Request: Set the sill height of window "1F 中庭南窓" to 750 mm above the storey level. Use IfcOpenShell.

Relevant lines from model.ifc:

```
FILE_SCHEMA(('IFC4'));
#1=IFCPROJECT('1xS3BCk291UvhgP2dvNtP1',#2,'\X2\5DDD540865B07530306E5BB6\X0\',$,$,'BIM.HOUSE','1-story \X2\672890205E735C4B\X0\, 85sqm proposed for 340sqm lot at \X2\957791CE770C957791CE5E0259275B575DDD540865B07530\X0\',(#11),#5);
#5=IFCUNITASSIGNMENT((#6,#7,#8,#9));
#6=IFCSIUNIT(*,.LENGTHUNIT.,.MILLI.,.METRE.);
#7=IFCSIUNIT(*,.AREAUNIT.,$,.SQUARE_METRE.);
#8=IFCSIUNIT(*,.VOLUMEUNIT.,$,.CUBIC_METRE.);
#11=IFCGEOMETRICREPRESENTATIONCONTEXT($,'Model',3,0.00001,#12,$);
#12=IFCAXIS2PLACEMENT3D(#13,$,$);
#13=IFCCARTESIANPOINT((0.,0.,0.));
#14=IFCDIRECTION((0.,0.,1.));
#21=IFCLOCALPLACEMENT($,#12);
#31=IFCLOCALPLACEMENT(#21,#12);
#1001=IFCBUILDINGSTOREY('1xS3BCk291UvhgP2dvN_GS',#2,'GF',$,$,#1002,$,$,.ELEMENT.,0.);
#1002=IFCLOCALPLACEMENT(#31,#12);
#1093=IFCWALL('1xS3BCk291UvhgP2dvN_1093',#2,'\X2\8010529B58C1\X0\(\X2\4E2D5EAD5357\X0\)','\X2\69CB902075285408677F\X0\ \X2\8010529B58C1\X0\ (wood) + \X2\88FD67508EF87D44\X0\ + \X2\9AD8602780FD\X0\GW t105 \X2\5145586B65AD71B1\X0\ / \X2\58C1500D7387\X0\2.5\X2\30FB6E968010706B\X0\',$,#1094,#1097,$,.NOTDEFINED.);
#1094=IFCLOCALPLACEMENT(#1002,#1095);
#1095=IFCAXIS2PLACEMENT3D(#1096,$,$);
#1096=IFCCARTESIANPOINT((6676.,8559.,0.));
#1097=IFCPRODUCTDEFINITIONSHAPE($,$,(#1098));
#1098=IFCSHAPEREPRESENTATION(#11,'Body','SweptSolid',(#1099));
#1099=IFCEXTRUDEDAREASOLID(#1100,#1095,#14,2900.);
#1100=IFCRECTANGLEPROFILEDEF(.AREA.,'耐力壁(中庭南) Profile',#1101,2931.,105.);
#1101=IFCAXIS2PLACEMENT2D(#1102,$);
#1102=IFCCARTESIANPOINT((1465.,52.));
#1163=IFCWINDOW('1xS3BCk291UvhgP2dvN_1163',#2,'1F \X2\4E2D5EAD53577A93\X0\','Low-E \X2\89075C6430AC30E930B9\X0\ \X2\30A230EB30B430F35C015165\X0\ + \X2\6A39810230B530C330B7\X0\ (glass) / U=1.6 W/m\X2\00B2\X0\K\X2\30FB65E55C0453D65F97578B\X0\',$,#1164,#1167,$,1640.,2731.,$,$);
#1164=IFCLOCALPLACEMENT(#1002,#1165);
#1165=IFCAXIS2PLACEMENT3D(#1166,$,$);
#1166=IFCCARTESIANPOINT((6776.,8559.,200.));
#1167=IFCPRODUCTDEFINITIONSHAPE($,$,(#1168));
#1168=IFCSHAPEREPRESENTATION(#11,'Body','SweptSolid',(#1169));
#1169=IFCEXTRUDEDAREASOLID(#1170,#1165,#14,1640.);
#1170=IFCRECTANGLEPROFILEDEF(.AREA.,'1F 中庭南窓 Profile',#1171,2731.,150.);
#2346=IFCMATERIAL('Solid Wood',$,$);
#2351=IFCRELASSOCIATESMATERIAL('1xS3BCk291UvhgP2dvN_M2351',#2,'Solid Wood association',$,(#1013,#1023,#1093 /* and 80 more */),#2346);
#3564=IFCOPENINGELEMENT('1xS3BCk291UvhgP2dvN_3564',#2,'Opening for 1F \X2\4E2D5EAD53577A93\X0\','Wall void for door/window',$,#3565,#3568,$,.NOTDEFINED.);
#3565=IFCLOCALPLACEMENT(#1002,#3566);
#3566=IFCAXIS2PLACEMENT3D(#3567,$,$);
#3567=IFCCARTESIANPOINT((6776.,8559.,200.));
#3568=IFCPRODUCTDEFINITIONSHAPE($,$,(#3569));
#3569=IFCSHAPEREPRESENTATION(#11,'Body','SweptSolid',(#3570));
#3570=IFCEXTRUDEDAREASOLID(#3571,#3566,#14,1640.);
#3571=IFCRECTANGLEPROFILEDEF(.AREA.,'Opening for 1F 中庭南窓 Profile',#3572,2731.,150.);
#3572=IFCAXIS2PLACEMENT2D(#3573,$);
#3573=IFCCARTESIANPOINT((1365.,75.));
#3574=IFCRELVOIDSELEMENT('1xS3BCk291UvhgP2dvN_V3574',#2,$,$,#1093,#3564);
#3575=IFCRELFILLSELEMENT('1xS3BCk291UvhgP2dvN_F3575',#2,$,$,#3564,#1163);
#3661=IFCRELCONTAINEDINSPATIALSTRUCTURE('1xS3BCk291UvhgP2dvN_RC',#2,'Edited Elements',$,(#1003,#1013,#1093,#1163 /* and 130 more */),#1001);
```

```python
import numpy as np
import ifcopenshell
import ifcopenshell.api.geometry
import ifcopenshell.geom
import ifcopenshell.util.element
import ifcopenshell.util.placement
import ifcopenshell.util.shape
import ifcopenshell.util.unit

model = ifcopenshell.open("model.ifc")
unit_scale = ifcopenshell.util.unit.calculate_unit_scale(model)

window = model.by_guid("1xS3BCk291UvhgP2dvN_1163")
opening = window.FillsVoids[0].RelatingOpeningElement
storey = ifcopenshell.util.element.get_container(window, ifc_class="IfcBuildingStorey")
level = ifcopenshell.util.placement.get_local_placement(storey.ObjectPlacement)[2, 3]

# The opening's origin need not be at the sill, so measure its lowest point.
shape = ifcopenshell.geom.create_shape(ifcopenshell.geom.settings(), opening)
bottom = ifcopenshell.util.shape.get_shape_bottom_elevation(shape, shape.geometry) / unit_scale
dz = level + 750.0 - bottom

shift = np.array([0.0, 0.0, dz])
# The window is not placed relative to its opening, so move both.
for product in (opening, window):
    matrix = ifcopenshell.util.placement.get_local_placement(product.ObjectPlacement)
    matrix[:3, 3] += shift
    ifcopenshell.api.geometry.edit_object_placement(model, product=product, matrix=matrix, is_si=False)

print(f"moved by {dz * unit_scale:+.3f} m")

model.write("model_updated.ifc")
```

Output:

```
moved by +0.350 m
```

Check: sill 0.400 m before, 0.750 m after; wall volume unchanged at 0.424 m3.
